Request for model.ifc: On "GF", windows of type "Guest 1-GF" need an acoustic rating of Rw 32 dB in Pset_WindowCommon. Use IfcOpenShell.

First a look at what the model holds.

```python
import ifcopenshell
import ifcopenshell.util.element

model = ifcopenshell.open("model.ifc")
print(model.schema)
storey = next(s for s in model.by_type("IfcBuildingStorey") if s.Name == "GF")
windows = [e for e in ifcopenshell.util.element.get_decomposition(storey) if e.is_a("IfcWindow")]
seen = {}
for e in windows:
    element_type = ifcopenshell.util.element.get_type(e)
    key = (element_type.Name if element_type != e and element_type else None, ifcopenshell.util.element.get_pset(e, "Pset_WindowCommon", "AcousticRating"))
    seen[key] = seen.get(key, 0) + 1
for (name, value), count in sorted(seen.items(), key=str):
    print(count, "x", name, "|", value)
```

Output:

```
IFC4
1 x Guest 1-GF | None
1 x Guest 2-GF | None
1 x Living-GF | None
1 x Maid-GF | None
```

```python
import ifcopenshell
import ifcopenshell.api.pset
import ifcopenshell.util.element

model = ifcopenshell.open("model.ifc")

storey = next(s for s in model.by_type("IfcBuildingStorey") if s.Name == "GF")
windows = [e for e in ifcopenshell.util.element.get_decomposition(storey) if e.is_a("IfcWindow")]

count = 0
for e in windows:
    element_type = ifcopenshell.util.element.get_type(e)
    if element_type in (None, e) or element_type.Name != "Guest 1-GF":
        continue
    # add_pset returns the element's existing set when there is one.
    pset = ifcopenshell.api.pset.add_pset(model, product=e, name="Pset_WindowCommon")
    ifcopenshell.api.pset.edit_pset(model, pset=pset, properties={"AcousticRating": "Rw 32 dB"})
    count += 1

print(count, "windows updated")

model.write("model_rev.ifc")
```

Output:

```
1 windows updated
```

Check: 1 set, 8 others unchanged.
